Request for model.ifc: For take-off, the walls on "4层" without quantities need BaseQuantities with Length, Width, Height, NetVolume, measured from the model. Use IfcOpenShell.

First a look at what the model holds.

```python
import ifcopenshell
import ifcopenshell.util.element
import ifcopenshell.util.unit

model = ifcopenshell.open("model.ifc")
print(model.schema)
for unit_type in ("LENGTHUNIT", "AREAUNIT", "VOLUMEUNIT"):
    print(unit_type, ifcopenshell.util.unit.calculate_unit_scale(model, unit_type))
storey = next(s for s in model.by_type("IfcBuildingStorey") if s.Name == "4层")
walls = [e for e in ifcopenshell.util.element.get_decomposition(storey) if e.is_a("IfcWall")]
for e in sorted(walls, key=lambda e: e.id()):
    print(e.id(), e.is_a(), e.Name, list(ifcopenshell.util.element.get_psets(e, qtos_only=True)), sep=" | ")
```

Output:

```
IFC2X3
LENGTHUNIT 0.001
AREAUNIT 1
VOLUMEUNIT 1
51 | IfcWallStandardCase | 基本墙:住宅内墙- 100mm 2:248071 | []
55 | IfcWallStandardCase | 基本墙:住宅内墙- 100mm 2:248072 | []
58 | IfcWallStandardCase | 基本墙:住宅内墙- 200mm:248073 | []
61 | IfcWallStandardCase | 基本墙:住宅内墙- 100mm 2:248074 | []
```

```python
import ifcopenshell
import ifcopenshell.api.pset
import ifcopenshell.geom
import ifcopenshell.util.element
import ifcopenshell.util.shape
import ifcopenshell.util.unit

model = ifcopenshell.open("model.ifc")
unit_scale = ifcopenshell.util.unit.calculate_unit_scale(model)
volume_scale = ifcopenshell.util.unit.calculate_unit_scale(model, "VOLUMEUNIT")
settings = ifcopenshell.geom.settings()

storey = next(s for s in model.by_type("IfcBuildingStorey") if s.Name == "4层")
walls = [e for e in ifcopenshell.util.element.get_decomposition(storey) if e.is_a("IfcWall")]

for e in sorted(walls, key=lambda e: e.id()):
    if ifcopenshell.util.element.get_psets(e, qtos_only=True, should_inherit=False):
        continue
    # Geometry comes back in metres, in the element's own axes.
    shape = ifcopenshell.geom.create_shape(settings, e)
    values = {
        "Length": ifcopenshell.util.shape.get_x(shape.geometry) / unit_scale,
        "Width": ifcopenshell.util.shape.get_y(shape.geometry) / unit_scale,
        "Height": ifcopenshell.util.shape.get_z(shape.geometry) / unit_scale,
        "NetVolume": ifcopenshell.util.shape.get_volume(shape.geometry) / volume_scale,
    }
    qto = ifcopenshell.api.pset.add_qto(model, product=e, name="BaseQuantities")
    ifcopenshell.api.pset.edit_qto(model, qto=qto, properties=values)
    print(e.id(), {k: round(v, 3) for k, v in values.items()})

model.write("model_edited.ifc")
```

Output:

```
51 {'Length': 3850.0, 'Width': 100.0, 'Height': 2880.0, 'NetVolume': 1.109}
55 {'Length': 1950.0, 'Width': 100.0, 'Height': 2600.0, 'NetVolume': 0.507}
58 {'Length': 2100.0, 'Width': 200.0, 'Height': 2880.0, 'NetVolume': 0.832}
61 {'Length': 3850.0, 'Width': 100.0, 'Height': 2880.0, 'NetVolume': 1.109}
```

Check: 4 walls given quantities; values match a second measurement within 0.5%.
